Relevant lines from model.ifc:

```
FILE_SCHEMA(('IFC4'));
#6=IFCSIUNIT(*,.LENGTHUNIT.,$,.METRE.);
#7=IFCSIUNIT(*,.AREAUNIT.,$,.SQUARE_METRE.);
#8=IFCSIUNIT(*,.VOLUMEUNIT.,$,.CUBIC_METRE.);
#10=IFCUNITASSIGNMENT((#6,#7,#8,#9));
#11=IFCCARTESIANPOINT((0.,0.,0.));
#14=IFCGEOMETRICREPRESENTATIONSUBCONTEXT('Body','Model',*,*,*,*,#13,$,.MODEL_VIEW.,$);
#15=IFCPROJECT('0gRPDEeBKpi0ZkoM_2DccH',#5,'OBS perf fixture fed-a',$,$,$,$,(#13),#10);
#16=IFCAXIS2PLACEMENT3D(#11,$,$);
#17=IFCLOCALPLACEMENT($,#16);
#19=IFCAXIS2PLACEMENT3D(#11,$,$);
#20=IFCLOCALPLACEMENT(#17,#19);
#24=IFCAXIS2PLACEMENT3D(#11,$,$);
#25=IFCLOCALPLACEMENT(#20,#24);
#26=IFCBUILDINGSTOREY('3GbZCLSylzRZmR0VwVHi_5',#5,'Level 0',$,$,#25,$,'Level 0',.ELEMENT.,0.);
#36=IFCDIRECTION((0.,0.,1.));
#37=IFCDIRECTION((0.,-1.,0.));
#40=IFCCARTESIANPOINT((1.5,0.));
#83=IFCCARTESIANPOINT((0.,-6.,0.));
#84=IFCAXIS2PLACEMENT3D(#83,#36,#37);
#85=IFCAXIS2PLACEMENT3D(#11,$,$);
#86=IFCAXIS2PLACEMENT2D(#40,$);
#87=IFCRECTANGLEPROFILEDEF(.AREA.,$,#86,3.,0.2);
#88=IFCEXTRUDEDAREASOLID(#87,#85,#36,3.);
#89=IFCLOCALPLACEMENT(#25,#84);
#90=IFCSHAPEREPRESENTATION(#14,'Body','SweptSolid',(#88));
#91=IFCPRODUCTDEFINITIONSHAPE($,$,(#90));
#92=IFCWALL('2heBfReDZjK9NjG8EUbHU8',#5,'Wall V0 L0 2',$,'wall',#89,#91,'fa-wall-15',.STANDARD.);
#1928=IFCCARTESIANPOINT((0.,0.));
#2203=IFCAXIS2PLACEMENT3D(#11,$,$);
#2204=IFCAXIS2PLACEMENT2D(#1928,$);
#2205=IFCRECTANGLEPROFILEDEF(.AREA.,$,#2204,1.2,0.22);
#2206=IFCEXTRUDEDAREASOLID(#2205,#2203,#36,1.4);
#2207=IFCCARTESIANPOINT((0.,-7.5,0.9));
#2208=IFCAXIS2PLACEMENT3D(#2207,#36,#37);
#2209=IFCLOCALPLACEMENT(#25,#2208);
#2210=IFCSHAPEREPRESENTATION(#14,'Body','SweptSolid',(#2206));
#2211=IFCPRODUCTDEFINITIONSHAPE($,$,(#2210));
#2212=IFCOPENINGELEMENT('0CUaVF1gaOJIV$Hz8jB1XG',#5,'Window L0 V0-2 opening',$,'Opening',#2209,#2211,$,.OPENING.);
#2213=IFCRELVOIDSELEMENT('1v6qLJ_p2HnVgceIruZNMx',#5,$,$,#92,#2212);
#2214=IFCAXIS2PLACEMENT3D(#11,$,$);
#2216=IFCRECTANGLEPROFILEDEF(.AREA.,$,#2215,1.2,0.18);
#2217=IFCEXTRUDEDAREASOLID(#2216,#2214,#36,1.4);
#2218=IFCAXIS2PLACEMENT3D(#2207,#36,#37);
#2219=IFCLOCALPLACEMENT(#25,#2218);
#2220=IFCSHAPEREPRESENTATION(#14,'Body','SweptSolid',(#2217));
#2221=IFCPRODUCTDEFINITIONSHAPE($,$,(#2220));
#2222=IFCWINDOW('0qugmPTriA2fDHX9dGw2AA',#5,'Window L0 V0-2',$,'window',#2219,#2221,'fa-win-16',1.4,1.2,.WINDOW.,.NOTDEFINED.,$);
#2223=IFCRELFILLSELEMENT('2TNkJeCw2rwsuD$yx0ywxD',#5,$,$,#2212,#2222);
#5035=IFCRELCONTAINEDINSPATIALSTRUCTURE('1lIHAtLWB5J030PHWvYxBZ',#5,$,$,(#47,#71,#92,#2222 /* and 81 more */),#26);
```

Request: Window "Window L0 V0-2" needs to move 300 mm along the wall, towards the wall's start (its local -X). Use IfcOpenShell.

```python
import ifcopenshell
import ifcopenshell.api.geometry
import ifcopenshell.util.placement

model = ifcopenshell.open("model.ifc")

window = model.by_guid("0qugmPTriA2fDHX9dGw2AA")
opening = window.FillsVoids[0].RelatingOpeningElement
wall = opening.VoidsElements[0].RelatingBuildingElement

wall_matrix = ifcopenshell.util.placement.get_local_placement(wall.ObjectPlacement)
shift = wall_matrix[:3, 0] * -0.3
before = ifcopenshell.util.placement.get_local_placement(window.ObjectPlacement)[:3, 3].copy()

# The window is not placed relative to its opening, so move both.
for product in (opening, window):
    matrix = ifcopenshell.util.placement.get_local_placement(product.ObjectPlacement)
    matrix[:3, 3] += shift
    ifcopenshell.api.geometry.edit_object_placement(model, product=product, matrix=matrix, is_si=False)

after = ifcopenshell.util.placement.get_local_placement(window.ObjectPlacement)[:3, 3]
print("window moved by", (after - before).round(3) + 0.0)

model.write("model_rev.ifc")
```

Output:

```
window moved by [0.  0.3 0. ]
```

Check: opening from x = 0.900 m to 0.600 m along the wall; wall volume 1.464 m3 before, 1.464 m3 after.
